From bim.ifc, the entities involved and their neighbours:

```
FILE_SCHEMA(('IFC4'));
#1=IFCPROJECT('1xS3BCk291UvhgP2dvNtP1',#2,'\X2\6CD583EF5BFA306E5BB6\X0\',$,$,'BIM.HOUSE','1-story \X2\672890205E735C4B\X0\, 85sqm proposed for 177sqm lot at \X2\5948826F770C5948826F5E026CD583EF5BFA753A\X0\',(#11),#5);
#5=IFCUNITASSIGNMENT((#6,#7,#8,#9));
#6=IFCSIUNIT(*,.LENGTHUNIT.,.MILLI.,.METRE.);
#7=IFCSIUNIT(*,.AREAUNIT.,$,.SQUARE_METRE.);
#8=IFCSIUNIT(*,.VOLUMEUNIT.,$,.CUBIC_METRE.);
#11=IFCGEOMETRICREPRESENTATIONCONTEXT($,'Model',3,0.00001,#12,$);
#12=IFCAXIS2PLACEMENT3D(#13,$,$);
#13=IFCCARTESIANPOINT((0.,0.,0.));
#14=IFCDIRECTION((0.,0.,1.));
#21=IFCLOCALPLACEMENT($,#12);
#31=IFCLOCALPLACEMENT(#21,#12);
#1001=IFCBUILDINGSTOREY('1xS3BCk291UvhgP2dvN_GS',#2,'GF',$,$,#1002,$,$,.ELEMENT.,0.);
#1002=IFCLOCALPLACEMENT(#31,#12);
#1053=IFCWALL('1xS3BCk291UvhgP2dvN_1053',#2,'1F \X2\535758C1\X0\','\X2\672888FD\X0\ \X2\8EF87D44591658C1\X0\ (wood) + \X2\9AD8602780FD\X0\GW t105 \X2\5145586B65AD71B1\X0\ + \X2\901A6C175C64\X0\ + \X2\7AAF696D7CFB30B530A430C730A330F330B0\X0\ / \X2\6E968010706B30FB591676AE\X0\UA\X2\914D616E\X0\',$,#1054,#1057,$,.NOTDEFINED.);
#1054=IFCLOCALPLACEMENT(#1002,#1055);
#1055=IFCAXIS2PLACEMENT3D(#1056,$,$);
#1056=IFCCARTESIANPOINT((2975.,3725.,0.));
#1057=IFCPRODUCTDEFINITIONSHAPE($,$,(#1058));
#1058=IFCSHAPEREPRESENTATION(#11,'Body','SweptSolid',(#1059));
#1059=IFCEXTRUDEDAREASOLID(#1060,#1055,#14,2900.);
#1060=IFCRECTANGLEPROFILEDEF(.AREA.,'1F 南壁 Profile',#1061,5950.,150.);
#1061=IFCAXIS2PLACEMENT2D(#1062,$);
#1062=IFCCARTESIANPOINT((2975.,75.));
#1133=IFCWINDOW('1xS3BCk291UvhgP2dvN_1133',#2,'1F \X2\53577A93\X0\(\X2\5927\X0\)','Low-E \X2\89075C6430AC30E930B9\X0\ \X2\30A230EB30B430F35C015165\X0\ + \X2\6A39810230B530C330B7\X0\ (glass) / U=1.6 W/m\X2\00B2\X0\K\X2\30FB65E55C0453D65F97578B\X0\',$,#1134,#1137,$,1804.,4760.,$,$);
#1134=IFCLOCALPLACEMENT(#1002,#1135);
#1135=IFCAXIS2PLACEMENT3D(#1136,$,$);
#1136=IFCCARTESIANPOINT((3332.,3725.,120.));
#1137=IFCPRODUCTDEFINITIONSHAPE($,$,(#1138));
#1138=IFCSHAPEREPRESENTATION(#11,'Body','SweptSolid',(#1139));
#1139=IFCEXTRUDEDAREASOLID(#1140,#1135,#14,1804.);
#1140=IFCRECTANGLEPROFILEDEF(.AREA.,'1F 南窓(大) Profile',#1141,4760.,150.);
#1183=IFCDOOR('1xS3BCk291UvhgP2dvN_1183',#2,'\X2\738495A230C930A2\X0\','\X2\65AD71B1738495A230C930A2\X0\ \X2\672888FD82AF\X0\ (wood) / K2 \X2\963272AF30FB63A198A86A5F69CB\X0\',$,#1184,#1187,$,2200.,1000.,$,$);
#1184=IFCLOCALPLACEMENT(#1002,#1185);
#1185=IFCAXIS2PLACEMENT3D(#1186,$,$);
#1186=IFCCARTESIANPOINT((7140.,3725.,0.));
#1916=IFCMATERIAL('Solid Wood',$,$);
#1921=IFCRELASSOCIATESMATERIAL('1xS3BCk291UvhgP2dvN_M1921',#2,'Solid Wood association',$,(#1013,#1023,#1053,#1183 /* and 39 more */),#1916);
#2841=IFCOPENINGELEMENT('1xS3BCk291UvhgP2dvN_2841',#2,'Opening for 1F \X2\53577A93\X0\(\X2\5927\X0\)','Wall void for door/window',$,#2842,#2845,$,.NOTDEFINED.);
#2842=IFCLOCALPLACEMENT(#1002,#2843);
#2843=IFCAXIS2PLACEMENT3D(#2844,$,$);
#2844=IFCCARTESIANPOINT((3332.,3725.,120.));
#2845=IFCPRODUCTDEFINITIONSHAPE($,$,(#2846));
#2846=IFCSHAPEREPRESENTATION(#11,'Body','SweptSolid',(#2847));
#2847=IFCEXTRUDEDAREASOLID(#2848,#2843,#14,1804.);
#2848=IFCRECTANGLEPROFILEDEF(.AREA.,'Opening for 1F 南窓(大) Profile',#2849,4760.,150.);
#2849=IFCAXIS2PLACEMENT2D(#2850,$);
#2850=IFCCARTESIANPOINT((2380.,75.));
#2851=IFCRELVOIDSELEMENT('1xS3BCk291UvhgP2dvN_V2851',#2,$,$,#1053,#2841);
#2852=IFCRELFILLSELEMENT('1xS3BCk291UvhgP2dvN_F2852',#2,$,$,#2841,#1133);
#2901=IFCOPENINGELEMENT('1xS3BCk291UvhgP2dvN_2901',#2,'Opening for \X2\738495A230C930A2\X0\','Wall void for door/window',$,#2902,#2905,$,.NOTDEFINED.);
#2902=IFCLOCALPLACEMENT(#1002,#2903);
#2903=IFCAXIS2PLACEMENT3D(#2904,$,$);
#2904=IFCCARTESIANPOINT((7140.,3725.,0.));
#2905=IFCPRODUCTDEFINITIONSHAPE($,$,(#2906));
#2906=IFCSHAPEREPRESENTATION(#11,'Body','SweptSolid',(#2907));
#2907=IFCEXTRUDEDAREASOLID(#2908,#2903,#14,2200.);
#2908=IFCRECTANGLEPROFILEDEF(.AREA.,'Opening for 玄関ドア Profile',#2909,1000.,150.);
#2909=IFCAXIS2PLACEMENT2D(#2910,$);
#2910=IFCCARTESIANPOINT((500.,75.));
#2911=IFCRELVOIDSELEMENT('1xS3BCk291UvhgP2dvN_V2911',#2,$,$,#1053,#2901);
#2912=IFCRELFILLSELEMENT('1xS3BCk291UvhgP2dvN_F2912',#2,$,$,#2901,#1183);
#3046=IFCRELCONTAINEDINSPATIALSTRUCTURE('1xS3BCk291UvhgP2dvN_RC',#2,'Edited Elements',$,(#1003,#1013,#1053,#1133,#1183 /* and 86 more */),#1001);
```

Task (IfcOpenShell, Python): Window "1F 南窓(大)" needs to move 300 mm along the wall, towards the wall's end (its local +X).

```python
import ifcopenshell
import ifcopenshell.api.geometry
import ifcopenshell.util.placement
import ifcopenshell.util.unit

model = ifcopenshell.open("bim.ifc")
unit_scale = ifcopenshell.util.unit.calculate_unit_scale(model)

window = model.by_id(1133)
opening = window.FillsVoids[0].RelatingOpeningElement
wall = opening.VoidsElements[0].RelatingBuildingElement

wall_matrix = ifcopenshell.util.placement.get_local_placement(wall.ObjectPlacement)
shift = wall_matrix[:3, 0] * 0.3 / unit_scale
before = ifcopenshell.util.placement.get_local_placement(window.ObjectPlacement)[:3, 3].copy()

# The window is not placed relative to its opening, so move both.
for product in (opening, window):
    matrix = ifcopenshell.util.placement.get_local_placement(product.ObjectPlacement)
    matrix[:3, 3] += shift
    ifcopenshell.api.geometry.edit_object_placement(model, product=product, matrix=matrix, is_si=False)

after = ifcopenshell.util.placement.get_local_placement(window.ObjectPlacement)[:3, 3]
print("window moved by", (after - before).round(3) + 0.0)

model.write("bim_updated.ifc")
```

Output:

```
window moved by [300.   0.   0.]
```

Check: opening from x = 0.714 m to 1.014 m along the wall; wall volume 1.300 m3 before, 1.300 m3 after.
